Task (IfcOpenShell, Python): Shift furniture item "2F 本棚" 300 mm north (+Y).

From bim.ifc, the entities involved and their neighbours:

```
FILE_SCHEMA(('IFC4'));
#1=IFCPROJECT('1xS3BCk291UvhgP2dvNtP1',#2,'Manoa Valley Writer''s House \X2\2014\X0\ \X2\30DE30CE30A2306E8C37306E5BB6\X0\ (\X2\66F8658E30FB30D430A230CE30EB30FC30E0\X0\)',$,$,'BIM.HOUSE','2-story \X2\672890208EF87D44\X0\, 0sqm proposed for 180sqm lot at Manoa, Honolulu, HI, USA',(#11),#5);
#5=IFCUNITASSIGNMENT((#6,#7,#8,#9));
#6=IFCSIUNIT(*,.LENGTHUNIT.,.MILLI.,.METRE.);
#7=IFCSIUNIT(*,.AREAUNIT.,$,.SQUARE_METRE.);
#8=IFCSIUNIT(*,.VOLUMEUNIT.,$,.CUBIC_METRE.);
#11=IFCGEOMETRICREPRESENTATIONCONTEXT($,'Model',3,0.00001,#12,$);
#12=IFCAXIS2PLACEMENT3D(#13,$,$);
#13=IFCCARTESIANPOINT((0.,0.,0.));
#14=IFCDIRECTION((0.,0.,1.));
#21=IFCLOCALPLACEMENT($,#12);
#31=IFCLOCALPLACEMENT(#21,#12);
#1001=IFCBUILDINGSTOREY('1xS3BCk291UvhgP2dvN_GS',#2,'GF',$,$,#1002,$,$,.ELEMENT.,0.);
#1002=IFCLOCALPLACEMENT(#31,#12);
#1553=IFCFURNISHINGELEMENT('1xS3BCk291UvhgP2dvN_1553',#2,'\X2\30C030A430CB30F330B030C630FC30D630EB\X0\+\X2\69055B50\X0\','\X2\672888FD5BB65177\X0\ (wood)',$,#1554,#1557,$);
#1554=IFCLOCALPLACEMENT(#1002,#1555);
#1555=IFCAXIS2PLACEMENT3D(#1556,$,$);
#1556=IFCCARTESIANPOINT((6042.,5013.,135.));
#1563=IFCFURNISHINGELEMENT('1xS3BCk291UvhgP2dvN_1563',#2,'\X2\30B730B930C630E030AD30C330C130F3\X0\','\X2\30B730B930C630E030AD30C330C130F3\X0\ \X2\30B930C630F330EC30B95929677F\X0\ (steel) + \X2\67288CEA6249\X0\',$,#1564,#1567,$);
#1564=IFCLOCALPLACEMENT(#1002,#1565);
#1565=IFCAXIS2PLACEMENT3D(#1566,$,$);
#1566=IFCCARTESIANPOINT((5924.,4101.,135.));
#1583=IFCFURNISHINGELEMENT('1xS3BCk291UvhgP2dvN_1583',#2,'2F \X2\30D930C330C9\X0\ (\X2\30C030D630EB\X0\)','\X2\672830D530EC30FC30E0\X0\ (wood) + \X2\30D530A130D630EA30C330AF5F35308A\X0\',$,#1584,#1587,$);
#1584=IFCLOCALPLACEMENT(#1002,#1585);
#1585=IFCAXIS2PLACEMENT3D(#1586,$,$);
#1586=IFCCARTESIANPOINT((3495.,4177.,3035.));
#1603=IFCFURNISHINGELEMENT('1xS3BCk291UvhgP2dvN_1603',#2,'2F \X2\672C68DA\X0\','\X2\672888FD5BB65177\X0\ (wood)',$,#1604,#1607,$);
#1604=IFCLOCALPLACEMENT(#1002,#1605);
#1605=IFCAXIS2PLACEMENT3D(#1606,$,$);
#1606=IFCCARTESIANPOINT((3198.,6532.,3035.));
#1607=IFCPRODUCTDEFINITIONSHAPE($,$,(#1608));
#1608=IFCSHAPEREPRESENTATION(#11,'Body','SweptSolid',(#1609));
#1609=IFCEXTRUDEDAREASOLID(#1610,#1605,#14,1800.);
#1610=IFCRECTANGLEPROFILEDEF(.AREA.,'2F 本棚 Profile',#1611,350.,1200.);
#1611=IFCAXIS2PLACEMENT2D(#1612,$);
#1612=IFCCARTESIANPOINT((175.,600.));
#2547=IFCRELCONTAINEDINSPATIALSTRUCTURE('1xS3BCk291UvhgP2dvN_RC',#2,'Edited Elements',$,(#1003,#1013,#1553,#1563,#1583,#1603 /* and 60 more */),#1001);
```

```python
import ifcopenshell
import ifcopenshell.api.geometry
import ifcopenshell.util.placement

model = ifcopenshell.open("bim.ifc")

item = model.by_guid("1xS3BCk291UvhgP2dvN_1603")
matrix = ifcopenshell.util.placement.get_local_placement(item.ObjectPlacement)
matrix[1, 3] += 300.0
ifcopenshell.api.geometry.edit_object_placement(model, product=item, matrix=matrix, is_si=False)

print(ifcopenshell.util.placement.get_local_placement(item.ObjectPlacement).round(3) + 0.0)

model.write("bim-out.ifc")
```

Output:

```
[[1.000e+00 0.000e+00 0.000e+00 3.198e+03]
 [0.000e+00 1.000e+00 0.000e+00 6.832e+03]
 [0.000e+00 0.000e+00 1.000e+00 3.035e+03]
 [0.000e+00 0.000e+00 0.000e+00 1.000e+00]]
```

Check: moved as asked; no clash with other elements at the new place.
